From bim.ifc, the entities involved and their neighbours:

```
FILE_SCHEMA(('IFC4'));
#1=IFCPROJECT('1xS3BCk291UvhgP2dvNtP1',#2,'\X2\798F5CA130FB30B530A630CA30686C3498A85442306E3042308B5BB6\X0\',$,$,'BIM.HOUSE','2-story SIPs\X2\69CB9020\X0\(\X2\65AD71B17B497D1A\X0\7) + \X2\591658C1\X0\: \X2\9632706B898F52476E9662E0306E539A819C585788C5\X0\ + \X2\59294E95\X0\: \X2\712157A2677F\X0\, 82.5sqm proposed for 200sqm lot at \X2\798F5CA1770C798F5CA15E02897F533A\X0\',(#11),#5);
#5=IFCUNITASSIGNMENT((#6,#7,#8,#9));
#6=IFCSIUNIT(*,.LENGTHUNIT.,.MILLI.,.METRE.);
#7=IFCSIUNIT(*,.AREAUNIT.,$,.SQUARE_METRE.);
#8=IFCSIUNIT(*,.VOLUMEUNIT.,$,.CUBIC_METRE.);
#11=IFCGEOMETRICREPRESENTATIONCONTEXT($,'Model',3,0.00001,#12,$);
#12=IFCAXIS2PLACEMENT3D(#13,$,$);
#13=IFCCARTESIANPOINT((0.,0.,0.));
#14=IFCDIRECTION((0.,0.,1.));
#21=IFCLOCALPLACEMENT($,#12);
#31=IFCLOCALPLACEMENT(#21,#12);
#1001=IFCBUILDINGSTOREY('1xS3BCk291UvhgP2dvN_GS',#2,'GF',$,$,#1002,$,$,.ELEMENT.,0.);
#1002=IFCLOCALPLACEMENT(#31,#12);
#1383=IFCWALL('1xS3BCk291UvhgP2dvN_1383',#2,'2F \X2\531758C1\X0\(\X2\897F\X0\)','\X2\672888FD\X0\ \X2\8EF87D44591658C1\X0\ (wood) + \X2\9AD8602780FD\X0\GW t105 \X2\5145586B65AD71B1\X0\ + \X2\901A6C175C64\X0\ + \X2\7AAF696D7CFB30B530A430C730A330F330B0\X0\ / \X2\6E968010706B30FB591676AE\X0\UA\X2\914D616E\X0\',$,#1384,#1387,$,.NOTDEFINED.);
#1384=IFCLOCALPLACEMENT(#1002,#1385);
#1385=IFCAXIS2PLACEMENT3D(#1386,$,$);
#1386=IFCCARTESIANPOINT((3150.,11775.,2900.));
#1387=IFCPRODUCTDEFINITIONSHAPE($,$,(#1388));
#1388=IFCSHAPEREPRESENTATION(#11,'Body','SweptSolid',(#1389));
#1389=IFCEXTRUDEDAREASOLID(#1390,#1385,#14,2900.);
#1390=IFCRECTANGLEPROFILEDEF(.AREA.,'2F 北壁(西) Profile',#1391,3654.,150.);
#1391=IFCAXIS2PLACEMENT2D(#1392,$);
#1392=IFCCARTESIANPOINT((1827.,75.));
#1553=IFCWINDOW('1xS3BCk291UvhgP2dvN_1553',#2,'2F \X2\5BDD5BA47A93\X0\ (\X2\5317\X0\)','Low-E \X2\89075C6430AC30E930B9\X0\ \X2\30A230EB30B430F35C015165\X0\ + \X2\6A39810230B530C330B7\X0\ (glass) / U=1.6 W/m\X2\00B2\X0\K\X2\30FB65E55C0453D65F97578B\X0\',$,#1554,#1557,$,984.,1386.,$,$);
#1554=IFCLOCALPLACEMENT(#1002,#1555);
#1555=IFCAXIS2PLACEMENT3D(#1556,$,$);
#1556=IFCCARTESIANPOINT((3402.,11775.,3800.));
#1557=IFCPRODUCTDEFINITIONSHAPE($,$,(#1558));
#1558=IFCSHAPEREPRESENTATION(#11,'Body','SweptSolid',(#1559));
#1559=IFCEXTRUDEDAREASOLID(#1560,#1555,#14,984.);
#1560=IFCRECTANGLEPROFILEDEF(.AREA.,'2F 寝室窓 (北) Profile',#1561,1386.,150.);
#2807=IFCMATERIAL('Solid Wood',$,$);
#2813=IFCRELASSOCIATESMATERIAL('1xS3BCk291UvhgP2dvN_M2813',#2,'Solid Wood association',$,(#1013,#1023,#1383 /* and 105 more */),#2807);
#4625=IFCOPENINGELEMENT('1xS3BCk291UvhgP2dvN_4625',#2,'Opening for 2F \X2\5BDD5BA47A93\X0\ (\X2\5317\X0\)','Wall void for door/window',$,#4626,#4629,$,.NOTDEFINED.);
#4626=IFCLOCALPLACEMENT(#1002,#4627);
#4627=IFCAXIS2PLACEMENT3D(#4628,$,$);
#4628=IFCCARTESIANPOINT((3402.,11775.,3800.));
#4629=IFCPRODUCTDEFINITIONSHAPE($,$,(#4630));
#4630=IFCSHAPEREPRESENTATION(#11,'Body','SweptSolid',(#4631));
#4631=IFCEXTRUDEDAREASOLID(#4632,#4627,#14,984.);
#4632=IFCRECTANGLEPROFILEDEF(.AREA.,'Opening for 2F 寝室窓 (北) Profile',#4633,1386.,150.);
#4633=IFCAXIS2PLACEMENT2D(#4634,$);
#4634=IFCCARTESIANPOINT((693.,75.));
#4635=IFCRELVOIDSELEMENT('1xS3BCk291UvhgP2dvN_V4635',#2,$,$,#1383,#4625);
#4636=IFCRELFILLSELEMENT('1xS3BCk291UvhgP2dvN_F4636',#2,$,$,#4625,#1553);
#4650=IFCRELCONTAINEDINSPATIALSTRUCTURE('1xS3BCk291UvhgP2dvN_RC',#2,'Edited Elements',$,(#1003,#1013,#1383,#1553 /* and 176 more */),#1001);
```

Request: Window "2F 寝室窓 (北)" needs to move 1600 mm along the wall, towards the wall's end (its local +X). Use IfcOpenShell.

```python
import ifcopenshell
import ifcopenshell.api.geometry
import ifcopenshell.util.placement
import ifcopenshell.util.unit

model = ifcopenshell.open("bim.ifc")
unit_scale = ifcopenshell.util.unit.calculate_unit_scale(model)

window = model.by_guid("1xS3BCk291UvhgP2dvN_1553")
opening = window.FillsVoids[0].RelatingOpeningElement
wall = opening.VoidsElements[0].RelatingBuildingElement

wall_matrix = ifcopenshell.util.placement.get_local_placement(wall.ObjectPlacement)
shift = wall_matrix[:3, 0] * 1.6 / unit_scale
before = ifcopenshell.util.placement.get_local_placement(window.ObjectPlacement)[:3, 3].copy()

# The window is not placed relative to its opening, so move both.
for product in (opening, window):
    matrix = ifcopenshell.util.placement.get_local_placement(product.ObjectPlacement)
    matrix[:3, 3] += shift
    ifcopenshell.api.geometry.edit_object_placement(model, product=product, matrix=matrix, is_si=False)

after = ifcopenshell.util.placement.get_local_placement(window.ObjectPlacement)[:3, 3]
print("window moved by", (after - before).round(3) + 0.0)

model.write("bim-out.ifc")
```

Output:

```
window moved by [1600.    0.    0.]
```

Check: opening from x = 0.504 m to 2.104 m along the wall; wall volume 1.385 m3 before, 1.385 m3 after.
